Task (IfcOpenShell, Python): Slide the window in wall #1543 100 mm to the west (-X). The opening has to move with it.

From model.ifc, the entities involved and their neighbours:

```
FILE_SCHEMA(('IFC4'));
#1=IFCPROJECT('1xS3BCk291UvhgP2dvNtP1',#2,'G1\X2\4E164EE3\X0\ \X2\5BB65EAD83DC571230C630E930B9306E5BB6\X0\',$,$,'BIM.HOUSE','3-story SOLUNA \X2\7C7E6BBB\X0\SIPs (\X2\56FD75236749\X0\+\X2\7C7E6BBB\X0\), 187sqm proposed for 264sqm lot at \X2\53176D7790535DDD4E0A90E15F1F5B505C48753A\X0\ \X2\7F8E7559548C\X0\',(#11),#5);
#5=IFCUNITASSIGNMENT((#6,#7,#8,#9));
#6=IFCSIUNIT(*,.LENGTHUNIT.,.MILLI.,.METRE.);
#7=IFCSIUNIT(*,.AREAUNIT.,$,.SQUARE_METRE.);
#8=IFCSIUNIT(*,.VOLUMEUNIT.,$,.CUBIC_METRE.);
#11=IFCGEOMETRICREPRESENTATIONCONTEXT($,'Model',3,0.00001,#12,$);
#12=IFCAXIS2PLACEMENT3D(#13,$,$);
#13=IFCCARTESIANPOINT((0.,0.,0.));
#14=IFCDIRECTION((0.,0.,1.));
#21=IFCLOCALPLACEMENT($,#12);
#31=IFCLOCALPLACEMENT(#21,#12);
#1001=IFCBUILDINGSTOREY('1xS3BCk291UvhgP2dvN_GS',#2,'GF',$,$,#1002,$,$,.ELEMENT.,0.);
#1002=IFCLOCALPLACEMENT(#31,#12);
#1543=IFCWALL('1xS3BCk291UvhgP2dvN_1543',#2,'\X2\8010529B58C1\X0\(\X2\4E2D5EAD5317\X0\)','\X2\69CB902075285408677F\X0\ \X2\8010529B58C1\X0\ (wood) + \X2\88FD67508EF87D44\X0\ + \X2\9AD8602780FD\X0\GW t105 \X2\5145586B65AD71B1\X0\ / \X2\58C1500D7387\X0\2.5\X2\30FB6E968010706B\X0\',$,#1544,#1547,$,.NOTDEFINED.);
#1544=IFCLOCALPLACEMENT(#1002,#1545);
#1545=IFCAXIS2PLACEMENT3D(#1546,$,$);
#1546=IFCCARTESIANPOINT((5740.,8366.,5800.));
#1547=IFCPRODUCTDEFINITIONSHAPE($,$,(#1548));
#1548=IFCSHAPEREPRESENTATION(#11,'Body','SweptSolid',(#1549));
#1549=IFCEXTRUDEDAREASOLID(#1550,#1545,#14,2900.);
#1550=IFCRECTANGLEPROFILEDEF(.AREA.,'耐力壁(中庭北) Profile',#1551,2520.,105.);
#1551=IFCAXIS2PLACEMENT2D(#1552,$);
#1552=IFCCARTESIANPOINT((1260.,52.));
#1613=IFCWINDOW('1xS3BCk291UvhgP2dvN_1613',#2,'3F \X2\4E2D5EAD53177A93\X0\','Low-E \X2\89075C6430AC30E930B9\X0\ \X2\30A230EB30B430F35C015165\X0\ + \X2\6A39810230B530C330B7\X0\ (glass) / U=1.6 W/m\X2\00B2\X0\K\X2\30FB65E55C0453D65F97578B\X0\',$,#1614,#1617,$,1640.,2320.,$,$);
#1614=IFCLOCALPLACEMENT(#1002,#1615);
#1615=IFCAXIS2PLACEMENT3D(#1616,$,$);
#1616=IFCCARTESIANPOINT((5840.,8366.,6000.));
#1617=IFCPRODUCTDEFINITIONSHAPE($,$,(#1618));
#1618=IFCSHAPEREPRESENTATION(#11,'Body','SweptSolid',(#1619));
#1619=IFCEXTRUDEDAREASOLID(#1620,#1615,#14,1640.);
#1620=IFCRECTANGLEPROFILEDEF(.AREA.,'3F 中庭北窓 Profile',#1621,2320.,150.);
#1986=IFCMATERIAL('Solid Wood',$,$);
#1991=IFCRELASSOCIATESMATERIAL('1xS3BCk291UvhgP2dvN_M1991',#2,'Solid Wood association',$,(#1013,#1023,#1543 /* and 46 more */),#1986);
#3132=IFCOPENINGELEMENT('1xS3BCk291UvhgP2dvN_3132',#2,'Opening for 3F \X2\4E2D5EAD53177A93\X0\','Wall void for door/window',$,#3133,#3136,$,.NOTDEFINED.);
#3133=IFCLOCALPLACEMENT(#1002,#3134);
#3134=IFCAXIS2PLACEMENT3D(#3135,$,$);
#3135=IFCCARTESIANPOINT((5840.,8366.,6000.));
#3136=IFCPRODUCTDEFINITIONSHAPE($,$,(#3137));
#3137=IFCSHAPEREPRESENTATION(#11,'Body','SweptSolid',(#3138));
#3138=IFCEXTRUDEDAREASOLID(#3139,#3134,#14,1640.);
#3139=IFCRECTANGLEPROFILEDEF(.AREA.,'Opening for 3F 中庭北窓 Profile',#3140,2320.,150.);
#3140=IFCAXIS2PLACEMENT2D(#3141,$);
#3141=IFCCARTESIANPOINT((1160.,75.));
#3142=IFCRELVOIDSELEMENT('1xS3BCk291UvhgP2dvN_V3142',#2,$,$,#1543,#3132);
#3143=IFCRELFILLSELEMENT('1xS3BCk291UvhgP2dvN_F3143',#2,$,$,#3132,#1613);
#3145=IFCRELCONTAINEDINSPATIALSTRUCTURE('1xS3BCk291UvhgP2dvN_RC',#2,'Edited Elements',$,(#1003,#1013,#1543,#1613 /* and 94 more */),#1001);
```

```python
import ifcopenshell
import ifcopenshell.api.geometry
import ifcopenshell.util.placement
import ifcopenshell.util.unit

model = ifcopenshell.open("model.ifc")
unit_scale = ifcopenshell.util.unit.calculate_unit_scale(model)

window = model.by_guid("1xS3BCk291UvhgP2dvN_1613")
opening = window.FillsVoids[0].RelatingOpeningElement
wall = opening.VoidsElements[0].RelatingBuildingElement

wall_matrix = ifcopenshell.util.placement.get_local_placement(wall.ObjectPlacement)
shift = wall_matrix[:3, 0] * -0.1 / unit_scale
before = ifcopenshell.util.placement.get_local_placement(window.ObjectPlacement)[:3, 3].copy()

# The window is not placed relative to its opening, so move both.
for product in (opening, window):
    matrix = ifcopenshell.util.placement.get_local_placement(product.ObjectPlacement)
    matrix[:3, 3] += shift
    ifcopenshell.api.geometry.edit_object_placement(model, product=product, matrix=matrix, is_si=False)

after = ifcopenshell.util.placement.get_local_placement(window.ObjectPlacement)[:3, 3]
print("window moved by", (after - before).round(3) + 0.0)

model.write("model_rev.ifc")
```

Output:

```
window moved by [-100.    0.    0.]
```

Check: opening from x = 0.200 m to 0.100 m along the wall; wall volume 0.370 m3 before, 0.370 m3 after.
